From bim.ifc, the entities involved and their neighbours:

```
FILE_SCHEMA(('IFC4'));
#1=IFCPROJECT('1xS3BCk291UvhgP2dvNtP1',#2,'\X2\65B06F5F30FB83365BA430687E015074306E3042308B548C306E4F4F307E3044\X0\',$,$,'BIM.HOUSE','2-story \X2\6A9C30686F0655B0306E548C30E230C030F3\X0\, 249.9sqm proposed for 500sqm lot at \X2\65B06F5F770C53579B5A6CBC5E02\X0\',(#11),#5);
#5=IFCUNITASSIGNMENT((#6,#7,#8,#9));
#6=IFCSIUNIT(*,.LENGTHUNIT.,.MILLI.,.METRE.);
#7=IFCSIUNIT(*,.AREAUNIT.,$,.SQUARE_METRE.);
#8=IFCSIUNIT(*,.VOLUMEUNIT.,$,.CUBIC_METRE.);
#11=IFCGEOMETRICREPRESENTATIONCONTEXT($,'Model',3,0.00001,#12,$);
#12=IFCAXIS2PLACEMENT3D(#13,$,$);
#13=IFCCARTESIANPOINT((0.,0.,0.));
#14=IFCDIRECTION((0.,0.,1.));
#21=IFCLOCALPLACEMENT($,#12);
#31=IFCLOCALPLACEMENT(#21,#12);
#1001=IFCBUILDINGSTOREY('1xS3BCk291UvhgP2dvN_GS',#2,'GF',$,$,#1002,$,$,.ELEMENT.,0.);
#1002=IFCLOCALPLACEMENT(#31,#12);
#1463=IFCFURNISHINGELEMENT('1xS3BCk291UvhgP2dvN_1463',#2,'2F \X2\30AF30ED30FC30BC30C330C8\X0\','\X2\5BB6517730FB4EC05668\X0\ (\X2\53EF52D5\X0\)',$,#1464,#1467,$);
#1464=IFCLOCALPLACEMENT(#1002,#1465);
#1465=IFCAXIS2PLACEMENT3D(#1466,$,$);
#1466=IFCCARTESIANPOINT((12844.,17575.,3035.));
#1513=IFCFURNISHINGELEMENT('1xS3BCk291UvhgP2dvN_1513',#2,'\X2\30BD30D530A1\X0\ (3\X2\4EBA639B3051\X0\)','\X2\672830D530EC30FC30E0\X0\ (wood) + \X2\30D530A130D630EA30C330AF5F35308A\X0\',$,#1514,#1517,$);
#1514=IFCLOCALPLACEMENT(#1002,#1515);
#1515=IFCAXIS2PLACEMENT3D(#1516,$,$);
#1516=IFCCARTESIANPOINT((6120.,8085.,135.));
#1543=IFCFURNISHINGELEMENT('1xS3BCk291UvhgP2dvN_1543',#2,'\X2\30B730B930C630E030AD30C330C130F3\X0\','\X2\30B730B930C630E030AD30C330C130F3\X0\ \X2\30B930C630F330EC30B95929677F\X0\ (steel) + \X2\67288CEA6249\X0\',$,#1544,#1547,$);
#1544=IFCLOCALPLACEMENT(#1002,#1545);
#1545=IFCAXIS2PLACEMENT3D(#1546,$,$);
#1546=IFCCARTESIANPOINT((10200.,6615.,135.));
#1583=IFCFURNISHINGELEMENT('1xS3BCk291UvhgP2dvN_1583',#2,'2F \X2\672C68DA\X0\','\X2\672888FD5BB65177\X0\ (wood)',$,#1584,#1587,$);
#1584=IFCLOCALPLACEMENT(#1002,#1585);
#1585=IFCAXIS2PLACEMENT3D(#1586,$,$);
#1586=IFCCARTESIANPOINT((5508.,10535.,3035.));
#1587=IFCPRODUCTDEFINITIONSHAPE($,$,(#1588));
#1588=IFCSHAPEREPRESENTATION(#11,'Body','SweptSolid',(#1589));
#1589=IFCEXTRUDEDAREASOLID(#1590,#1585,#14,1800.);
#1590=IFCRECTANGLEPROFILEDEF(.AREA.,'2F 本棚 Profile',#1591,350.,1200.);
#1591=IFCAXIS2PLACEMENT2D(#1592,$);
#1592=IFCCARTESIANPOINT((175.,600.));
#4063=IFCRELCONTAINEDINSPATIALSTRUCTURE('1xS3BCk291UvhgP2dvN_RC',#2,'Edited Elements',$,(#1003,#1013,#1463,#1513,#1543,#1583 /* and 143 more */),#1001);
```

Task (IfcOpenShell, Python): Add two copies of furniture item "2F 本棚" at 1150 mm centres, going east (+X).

```python
import numpy as np
import ifcopenshell
import ifcopenshell.api.geometry
import ifcopenshell.api.root
import ifcopenshell.util.element
import ifcopenshell.util.placement
import ifcopenshell.util.unit

model = ifcopenshell.open("bim.ifc")
unit_scale = ifcopenshell.util.unit.calculate_unit_scale(model)


def reuse_history(source, copy):
    """copy_class also copies each property set's owner history, people and application; keep the originals."""
    for rel in copy.IsDefinedBy:
        if rel.is_a("IfcRelDefinesByProperties") and (history := rel.RelatingPropertyDefinition.OwnerHistory):
            rel.RelatingPropertyDefinition.OwnerHistory = source.OwnerHistory
            ifcopenshell.util.element.remove_deep2(model, history)


source = model.by_guid("1xS3BCk291UvhgP2dvN_1583")
base = ifcopenshell.util.placement.get_local_placement(source.ObjectPlacement)
step = np.array([1.0, 0.0, 0.0]) * 1.15 / unit_scale

for i in range(1, 3):
    copy = ifcopenshell.api.root.copy_class(model, product=source)
    copy.Representation = ifcopenshell.util.element.copy_deep(
        model, source.Representation, exclude=["IfcGeometricRepresentationContext", "IfcRepresentationMap"]
    )
    reuse_history(source, copy)
    matrix = base.copy()
    matrix[:3, 3] += i * step
    print("added at", matrix[:3, 3].round(3) + 0.0)
    ifcopenshell.api.geometry.edit_object_placement(model, product=copy, matrix=matrix, is_si=False)

model.write("bim_v2.ifc")
```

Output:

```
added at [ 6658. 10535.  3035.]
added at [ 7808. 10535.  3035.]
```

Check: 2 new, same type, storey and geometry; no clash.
